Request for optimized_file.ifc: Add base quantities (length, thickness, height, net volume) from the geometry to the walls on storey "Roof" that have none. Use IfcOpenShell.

First a look at what the model holds.

```python
import ifcopenshell
import ifcopenshell.util.element
import ifcopenshell.util.unit

model = ifcopenshell.open("optimized_file.ifc")
print(model.schema)
for unit_type in ("LENGTHUNIT", "AREAUNIT", "VOLUMEUNIT"):
    print(unit_type, ifcopenshell.util.unit.calculate_unit_scale(model, unit_type))
storey = next(s for s in model.by_type("IfcBuildingStorey") if s.Name == "Roof")
walls = [e for e in ifcopenshell.util.element.get_decomposition(storey) if e.is_a("IfcWall")]
for e in sorted(walls, key=lambda e: e.id()):
    print(e.id(), e.is_a(), e.Name, list(ifcopenshell.util.element.get_psets(e, qtos_only=True)), sep=" | ")
```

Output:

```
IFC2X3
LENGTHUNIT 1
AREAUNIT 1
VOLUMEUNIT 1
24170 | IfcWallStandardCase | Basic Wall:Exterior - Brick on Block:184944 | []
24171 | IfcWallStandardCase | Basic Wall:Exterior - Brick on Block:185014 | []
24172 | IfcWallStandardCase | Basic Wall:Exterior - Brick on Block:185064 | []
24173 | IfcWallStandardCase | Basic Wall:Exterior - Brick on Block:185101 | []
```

```python
import ifcopenshell
import ifcopenshell.api.pset
import ifcopenshell.geom
import ifcopenshell.util.element
import ifcopenshell.util.shape
import ifcopenshell.util.unit

model = ifcopenshell.open("optimized_file.ifc")
unit_scale = ifcopenshell.util.unit.calculate_unit_scale(model)
volume_scale = ifcopenshell.util.unit.calculate_unit_scale(model, "VOLUMEUNIT")
settings = ifcopenshell.geom.settings()

storey = next(s for s in model.by_type("IfcBuildingStorey") if s.Name == "Roof")
walls = [e for e in ifcopenshell.util.element.get_decomposition(storey) if e.is_a("IfcWall")]

for e in sorted(walls, key=lambda e: e.id()):
    if ifcopenshell.util.element.get_psets(e, qtos_only=True, should_inherit=False):
        continue
    # Geometry comes back in metres, in the element's own axes.
    shape = ifcopenshell.geom.create_shape(settings, e)
    values = {
        "Length": ifcopenshell.util.shape.get_x(shape.geometry) / unit_scale,
        "Width": ifcopenshell.util.shape.get_y(shape.geometry) / unit_scale,
        "Height": ifcopenshell.util.shape.get_z(shape.geometry) / unit_scale,
        "NetVolume": ifcopenshell.util.shape.get_volume(shape.geometry) / volume_scale,
    }
    qto = ifcopenshell.api.pset.add_qto(model, product=e, name="BaseQuantities")
    ifcopenshell.api.pset.edit_qto(model, qto=qto, properties=values)
    print(e.id(), {k: round(v, 3) for k, v in values.items()})

model.write("optimized_file_updated.ifc")
```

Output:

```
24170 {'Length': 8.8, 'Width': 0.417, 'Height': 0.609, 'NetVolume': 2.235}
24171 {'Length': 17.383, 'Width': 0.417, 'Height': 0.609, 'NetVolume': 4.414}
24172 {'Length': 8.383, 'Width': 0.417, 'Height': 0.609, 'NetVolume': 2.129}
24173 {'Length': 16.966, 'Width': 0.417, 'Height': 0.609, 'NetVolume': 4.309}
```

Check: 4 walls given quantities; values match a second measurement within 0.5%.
